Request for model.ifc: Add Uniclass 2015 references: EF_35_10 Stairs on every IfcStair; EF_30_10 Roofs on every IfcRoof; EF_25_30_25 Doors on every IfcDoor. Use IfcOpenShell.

First a look at what the model holds.

```python
import ifcopenshell

model = ifcopenshell.open("model.ifc")
print(model.schema)
print("classifications:", [c.Name for c in model.by_type("IfcClassification")])
for ifc_class in ("IfcDoor", "IfcRoof", "IfcStair", "IfcWall", "IfcWindow"):
    print(ifc_class, len(model.by_type(ifc_class)))
```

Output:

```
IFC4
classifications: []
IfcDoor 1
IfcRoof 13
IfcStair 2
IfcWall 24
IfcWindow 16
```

```python
import ifcopenshell
import ifcopenshell.api.classification

model = ifcopenshell.open("model.ifc")

system = ifcopenshell.api.classification.add_classification(model, classification="Uniclass 2015")

codes = {
    "IfcStair": ("EF_35_10", "Stairs"),
    "IfcRoof": ("EF_30_10", "Roofs"),
    "IfcDoor": ("EF_25_30_25", "Doors"),
}
for ifc_class, (code, name) in codes.items():
    products = model.by_type(ifc_class)
    ifcopenshell.api.classification.add_reference(
        model, products=products, classification=system, identification=code, name=name
    )
    print(code, len(products))

model.write("model_updated.ifc")
```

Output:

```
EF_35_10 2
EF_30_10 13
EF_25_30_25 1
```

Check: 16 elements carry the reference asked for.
